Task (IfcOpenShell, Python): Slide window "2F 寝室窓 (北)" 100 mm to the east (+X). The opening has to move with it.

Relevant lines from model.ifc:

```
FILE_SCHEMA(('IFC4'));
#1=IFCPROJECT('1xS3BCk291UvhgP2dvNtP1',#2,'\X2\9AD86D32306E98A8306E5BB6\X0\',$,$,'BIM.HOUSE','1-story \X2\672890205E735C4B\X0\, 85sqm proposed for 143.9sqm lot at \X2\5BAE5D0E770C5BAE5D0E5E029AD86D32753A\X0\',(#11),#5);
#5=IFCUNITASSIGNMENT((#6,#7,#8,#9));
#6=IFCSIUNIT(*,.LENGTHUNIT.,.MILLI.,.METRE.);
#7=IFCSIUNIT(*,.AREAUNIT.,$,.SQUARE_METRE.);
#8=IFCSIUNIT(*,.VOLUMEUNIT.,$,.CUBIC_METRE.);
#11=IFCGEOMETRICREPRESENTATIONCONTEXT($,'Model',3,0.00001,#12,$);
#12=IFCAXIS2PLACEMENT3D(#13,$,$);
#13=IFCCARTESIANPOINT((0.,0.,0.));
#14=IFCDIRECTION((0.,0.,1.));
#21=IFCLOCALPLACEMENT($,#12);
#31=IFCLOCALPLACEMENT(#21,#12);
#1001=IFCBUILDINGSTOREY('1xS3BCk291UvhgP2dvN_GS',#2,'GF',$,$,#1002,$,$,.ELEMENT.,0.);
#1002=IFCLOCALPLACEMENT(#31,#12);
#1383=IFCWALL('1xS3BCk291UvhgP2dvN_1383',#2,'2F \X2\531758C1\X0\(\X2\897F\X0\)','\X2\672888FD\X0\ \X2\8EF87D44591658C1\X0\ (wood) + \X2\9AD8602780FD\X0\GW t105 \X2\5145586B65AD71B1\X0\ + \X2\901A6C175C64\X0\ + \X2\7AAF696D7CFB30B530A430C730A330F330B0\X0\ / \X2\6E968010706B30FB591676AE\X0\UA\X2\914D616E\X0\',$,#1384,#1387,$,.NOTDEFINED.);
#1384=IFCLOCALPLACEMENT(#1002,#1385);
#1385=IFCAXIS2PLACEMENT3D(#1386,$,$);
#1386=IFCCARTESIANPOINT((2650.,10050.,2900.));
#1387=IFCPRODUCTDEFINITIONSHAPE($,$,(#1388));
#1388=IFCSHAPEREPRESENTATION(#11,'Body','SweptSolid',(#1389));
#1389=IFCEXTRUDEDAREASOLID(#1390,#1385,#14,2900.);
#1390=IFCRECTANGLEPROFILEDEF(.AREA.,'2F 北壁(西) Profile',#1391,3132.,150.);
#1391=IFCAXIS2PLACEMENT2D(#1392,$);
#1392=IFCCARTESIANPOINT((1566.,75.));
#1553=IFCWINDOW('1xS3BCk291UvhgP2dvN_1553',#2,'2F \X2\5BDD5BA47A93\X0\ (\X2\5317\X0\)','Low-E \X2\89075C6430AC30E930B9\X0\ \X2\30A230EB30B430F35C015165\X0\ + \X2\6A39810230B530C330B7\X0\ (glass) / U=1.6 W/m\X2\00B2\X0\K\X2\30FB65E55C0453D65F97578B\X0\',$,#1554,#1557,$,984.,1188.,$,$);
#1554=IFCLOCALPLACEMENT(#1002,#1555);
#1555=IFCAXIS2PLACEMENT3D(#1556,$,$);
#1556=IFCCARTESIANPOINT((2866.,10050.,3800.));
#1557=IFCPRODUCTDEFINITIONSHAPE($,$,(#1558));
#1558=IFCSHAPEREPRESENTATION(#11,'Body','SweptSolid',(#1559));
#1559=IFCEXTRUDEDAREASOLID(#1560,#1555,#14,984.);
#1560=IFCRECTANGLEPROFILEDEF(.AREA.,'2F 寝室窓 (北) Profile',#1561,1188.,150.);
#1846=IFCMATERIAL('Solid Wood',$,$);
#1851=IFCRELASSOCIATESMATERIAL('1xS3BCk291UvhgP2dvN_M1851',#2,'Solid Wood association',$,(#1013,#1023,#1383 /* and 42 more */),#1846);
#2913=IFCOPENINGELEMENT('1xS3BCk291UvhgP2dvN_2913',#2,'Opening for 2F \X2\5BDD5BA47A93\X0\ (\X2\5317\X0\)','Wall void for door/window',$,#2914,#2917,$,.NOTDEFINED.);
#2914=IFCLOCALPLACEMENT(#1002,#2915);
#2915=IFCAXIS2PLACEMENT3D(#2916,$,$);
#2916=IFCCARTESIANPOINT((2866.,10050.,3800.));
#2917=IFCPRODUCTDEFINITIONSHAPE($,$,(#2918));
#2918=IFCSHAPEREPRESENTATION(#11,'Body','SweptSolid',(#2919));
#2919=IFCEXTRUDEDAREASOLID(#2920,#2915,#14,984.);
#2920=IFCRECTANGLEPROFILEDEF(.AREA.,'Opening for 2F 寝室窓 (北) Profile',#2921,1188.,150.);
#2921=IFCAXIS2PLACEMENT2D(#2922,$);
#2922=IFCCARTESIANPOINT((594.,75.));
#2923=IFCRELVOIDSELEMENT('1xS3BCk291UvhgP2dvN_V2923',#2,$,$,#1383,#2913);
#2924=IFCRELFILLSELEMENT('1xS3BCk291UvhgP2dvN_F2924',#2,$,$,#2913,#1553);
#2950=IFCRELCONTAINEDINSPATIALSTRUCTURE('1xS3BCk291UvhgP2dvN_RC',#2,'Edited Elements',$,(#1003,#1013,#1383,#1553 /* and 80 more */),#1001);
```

```python
import ifcopenshell
import ifcopenshell.api.geometry
import ifcopenshell.util.placement

model = ifcopenshell.open("model.ifc")

window = model.by_id(1553)
opening = window.FillsVoids[0].RelatingOpeningElement
wall = opening.VoidsElements[0].RelatingBuildingElement

wall_matrix = ifcopenshell.util.placement.get_local_placement(wall.ObjectPlacement)
shift = wall_matrix[:3, 0] * 100.0
before = ifcopenshell.util.placement.get_local_placement(window.ObjectPlacement)[:3, 3].copy()

# The window is not placed relative to its opening, so move both.
for product in (opening, window):
    matrix = ifcopenshell.util.placement.get_local_placement(product.ObjectPlacement)
    matrix[:3, 3] += shift
    ifcopenshell.api.geometry.edit_object_placement(model, product=product, matrix=matrix, is_si=False)

after = ifcopenshell.util.placement.get_local_placement(window.ObjectPlacement)[:3, 3]
print("window moved by", (after - before).round(3) + 0.0)

model.write("model_edited.ifc")
```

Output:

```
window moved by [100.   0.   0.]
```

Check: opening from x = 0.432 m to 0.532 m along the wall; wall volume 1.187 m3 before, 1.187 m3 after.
